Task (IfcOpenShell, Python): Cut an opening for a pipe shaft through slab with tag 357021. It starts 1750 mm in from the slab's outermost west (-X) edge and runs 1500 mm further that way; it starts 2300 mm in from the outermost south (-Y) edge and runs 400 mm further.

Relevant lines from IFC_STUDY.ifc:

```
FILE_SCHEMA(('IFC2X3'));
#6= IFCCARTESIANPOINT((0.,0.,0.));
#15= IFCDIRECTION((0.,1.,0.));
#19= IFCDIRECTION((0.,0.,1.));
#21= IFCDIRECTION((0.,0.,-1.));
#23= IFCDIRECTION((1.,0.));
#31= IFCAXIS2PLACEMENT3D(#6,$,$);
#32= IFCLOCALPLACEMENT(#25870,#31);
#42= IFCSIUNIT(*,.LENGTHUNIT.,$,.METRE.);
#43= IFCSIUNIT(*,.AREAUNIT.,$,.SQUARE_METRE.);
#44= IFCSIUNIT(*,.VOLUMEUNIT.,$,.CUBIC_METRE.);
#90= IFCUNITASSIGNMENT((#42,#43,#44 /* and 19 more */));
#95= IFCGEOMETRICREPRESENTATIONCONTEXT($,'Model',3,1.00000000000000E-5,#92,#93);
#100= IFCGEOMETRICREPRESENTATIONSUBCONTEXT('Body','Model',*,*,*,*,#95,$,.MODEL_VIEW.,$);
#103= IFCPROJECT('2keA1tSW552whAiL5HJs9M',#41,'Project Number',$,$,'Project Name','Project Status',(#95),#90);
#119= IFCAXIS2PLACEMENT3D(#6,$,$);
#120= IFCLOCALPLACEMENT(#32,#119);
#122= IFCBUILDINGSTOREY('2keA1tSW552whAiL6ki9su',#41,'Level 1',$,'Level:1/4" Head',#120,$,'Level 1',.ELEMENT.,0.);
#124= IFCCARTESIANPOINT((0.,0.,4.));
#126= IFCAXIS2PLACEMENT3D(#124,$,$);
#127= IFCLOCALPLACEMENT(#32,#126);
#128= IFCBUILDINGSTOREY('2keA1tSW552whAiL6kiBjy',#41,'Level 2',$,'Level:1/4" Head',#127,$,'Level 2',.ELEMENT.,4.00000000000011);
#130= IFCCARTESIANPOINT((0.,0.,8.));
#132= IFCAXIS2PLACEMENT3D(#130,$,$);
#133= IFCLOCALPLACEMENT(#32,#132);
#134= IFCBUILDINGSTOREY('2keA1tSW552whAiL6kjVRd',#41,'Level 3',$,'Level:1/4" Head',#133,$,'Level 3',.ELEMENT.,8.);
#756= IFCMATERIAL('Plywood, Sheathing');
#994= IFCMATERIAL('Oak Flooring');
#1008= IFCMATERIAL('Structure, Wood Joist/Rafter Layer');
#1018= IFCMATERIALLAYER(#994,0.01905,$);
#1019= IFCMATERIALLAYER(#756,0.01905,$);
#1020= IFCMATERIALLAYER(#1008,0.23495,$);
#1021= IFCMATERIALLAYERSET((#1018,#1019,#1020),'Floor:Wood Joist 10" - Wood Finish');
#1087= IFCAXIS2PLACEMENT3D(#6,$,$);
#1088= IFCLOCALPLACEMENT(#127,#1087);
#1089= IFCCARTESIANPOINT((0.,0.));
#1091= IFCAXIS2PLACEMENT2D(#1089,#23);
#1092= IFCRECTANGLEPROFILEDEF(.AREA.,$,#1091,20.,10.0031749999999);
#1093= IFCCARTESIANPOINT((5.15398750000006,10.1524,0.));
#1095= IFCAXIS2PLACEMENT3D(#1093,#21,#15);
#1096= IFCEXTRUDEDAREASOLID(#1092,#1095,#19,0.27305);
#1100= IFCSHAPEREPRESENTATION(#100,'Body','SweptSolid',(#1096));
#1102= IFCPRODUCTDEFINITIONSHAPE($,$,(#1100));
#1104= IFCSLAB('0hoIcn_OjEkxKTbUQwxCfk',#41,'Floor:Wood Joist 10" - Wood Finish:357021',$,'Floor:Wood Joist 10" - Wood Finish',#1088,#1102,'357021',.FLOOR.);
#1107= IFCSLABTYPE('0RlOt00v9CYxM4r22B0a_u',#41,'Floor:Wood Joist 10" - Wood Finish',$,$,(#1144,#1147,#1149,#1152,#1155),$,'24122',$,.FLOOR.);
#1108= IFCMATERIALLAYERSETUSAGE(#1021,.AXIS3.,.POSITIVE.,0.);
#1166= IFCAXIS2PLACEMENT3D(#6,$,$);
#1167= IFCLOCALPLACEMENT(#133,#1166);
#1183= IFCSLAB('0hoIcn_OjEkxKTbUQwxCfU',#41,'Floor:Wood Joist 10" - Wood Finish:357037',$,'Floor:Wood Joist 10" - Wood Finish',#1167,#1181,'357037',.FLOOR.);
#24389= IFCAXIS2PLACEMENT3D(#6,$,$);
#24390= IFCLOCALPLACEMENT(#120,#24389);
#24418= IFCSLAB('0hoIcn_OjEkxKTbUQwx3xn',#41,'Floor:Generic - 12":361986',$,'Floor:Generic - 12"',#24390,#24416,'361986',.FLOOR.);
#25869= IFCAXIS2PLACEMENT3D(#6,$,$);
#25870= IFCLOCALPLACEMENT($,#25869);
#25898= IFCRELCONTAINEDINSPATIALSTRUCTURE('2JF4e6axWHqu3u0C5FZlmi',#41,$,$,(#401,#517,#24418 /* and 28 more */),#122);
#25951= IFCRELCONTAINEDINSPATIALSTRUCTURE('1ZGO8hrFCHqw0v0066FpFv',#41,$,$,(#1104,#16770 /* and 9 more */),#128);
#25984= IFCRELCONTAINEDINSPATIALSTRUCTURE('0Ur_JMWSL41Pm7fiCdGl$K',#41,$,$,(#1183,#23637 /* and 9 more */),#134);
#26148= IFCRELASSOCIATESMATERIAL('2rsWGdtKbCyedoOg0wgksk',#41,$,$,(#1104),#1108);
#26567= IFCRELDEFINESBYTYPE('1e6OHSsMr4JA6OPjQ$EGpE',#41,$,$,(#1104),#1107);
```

```python
import numpy as np
import ifcopenshell
import ifcopenshell.api.feature
import ifcopenshell.api.geometry
import ifcopenshell.api.root
import ifcopenshell.geom
import ifcopenshell.util.placement
import ifcopenshell.util.representation
import ifcopenshell.util.shape
import ifcopenshell.util.unit

model = ifcopenshell.open("IFC_STUDY.ifc")
unit_scale = ifcopenshell.util.unit.calculate_unit_scale(model)
settings = ifcopenshell.geom.settings()


def volume(element):
    """Net volume in cubic metres, openings subtracted."""
    shape = ifcopenshell.geom.create_shape(settings, element)
    return ifcopenshell.util.shape.get_volume(shape.geometry)


slab = model.by_guid("0hoIcn_OjEkxKTbUQwxCfk")
before = volume(slab)

# Extent in the slab's own axes, in metres. The edges named are its -X and -Y sides.
slab_shape = ifcopenshell.geom.create_shape(settings, slab)
vertices = ifcopenshell.util.shape.get_vertices(slab_shape.geometry)
x_min, y_min, bottom = vertices.min(axis=0)
top = vertices[:, 2].max()

opening = ifcopenshell.api.root.create_entity(model, ifc_class="IfcOpeningElement", name="Pipe shaft opening")
context = ifcopenshell.util.representation.get_context(model, "Model", "Body", "MODEL_VIEW")
width, depth = 1.5, 0.4
outline = [(0.0, 0.0), (width, 0.0), (width, depth), (0.0, depth), (0.0, 0.0)]
# Overshoot both faces by 50 mm so the cut is clean.
shape = ifcopenshell.api.geometry.add_slab_representation(
    model, context=context, depth=top - bottom + 0.1, polyline=outline
)
ifcopenshell.api.geometry.assign_representation(model, product=opening, representation=shape)

matrix = ifcopenshell.util.placement.get_local_placement(slab.ObjectPlacement)
matrix[:, 3] = matrix @ np.append(np.array([x_min + 1.75, y_min + 2.3, bottom - 0.05]) / unit_scale, 1.0)
ifcopenshell.api.geometry.edit_object_placement(model, product=opening, matrix=matrix, is_si=False)
ifcopenshell.api.feature.add_feature(model, feature=opening, element=slab)

after = volume(slab)

print(f"slab volume {before:.3f} -> {after:.3f} m3")

model.write("IFC_STUDY_rev.ifc")
```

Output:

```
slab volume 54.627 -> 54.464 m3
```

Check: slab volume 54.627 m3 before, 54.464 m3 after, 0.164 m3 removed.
